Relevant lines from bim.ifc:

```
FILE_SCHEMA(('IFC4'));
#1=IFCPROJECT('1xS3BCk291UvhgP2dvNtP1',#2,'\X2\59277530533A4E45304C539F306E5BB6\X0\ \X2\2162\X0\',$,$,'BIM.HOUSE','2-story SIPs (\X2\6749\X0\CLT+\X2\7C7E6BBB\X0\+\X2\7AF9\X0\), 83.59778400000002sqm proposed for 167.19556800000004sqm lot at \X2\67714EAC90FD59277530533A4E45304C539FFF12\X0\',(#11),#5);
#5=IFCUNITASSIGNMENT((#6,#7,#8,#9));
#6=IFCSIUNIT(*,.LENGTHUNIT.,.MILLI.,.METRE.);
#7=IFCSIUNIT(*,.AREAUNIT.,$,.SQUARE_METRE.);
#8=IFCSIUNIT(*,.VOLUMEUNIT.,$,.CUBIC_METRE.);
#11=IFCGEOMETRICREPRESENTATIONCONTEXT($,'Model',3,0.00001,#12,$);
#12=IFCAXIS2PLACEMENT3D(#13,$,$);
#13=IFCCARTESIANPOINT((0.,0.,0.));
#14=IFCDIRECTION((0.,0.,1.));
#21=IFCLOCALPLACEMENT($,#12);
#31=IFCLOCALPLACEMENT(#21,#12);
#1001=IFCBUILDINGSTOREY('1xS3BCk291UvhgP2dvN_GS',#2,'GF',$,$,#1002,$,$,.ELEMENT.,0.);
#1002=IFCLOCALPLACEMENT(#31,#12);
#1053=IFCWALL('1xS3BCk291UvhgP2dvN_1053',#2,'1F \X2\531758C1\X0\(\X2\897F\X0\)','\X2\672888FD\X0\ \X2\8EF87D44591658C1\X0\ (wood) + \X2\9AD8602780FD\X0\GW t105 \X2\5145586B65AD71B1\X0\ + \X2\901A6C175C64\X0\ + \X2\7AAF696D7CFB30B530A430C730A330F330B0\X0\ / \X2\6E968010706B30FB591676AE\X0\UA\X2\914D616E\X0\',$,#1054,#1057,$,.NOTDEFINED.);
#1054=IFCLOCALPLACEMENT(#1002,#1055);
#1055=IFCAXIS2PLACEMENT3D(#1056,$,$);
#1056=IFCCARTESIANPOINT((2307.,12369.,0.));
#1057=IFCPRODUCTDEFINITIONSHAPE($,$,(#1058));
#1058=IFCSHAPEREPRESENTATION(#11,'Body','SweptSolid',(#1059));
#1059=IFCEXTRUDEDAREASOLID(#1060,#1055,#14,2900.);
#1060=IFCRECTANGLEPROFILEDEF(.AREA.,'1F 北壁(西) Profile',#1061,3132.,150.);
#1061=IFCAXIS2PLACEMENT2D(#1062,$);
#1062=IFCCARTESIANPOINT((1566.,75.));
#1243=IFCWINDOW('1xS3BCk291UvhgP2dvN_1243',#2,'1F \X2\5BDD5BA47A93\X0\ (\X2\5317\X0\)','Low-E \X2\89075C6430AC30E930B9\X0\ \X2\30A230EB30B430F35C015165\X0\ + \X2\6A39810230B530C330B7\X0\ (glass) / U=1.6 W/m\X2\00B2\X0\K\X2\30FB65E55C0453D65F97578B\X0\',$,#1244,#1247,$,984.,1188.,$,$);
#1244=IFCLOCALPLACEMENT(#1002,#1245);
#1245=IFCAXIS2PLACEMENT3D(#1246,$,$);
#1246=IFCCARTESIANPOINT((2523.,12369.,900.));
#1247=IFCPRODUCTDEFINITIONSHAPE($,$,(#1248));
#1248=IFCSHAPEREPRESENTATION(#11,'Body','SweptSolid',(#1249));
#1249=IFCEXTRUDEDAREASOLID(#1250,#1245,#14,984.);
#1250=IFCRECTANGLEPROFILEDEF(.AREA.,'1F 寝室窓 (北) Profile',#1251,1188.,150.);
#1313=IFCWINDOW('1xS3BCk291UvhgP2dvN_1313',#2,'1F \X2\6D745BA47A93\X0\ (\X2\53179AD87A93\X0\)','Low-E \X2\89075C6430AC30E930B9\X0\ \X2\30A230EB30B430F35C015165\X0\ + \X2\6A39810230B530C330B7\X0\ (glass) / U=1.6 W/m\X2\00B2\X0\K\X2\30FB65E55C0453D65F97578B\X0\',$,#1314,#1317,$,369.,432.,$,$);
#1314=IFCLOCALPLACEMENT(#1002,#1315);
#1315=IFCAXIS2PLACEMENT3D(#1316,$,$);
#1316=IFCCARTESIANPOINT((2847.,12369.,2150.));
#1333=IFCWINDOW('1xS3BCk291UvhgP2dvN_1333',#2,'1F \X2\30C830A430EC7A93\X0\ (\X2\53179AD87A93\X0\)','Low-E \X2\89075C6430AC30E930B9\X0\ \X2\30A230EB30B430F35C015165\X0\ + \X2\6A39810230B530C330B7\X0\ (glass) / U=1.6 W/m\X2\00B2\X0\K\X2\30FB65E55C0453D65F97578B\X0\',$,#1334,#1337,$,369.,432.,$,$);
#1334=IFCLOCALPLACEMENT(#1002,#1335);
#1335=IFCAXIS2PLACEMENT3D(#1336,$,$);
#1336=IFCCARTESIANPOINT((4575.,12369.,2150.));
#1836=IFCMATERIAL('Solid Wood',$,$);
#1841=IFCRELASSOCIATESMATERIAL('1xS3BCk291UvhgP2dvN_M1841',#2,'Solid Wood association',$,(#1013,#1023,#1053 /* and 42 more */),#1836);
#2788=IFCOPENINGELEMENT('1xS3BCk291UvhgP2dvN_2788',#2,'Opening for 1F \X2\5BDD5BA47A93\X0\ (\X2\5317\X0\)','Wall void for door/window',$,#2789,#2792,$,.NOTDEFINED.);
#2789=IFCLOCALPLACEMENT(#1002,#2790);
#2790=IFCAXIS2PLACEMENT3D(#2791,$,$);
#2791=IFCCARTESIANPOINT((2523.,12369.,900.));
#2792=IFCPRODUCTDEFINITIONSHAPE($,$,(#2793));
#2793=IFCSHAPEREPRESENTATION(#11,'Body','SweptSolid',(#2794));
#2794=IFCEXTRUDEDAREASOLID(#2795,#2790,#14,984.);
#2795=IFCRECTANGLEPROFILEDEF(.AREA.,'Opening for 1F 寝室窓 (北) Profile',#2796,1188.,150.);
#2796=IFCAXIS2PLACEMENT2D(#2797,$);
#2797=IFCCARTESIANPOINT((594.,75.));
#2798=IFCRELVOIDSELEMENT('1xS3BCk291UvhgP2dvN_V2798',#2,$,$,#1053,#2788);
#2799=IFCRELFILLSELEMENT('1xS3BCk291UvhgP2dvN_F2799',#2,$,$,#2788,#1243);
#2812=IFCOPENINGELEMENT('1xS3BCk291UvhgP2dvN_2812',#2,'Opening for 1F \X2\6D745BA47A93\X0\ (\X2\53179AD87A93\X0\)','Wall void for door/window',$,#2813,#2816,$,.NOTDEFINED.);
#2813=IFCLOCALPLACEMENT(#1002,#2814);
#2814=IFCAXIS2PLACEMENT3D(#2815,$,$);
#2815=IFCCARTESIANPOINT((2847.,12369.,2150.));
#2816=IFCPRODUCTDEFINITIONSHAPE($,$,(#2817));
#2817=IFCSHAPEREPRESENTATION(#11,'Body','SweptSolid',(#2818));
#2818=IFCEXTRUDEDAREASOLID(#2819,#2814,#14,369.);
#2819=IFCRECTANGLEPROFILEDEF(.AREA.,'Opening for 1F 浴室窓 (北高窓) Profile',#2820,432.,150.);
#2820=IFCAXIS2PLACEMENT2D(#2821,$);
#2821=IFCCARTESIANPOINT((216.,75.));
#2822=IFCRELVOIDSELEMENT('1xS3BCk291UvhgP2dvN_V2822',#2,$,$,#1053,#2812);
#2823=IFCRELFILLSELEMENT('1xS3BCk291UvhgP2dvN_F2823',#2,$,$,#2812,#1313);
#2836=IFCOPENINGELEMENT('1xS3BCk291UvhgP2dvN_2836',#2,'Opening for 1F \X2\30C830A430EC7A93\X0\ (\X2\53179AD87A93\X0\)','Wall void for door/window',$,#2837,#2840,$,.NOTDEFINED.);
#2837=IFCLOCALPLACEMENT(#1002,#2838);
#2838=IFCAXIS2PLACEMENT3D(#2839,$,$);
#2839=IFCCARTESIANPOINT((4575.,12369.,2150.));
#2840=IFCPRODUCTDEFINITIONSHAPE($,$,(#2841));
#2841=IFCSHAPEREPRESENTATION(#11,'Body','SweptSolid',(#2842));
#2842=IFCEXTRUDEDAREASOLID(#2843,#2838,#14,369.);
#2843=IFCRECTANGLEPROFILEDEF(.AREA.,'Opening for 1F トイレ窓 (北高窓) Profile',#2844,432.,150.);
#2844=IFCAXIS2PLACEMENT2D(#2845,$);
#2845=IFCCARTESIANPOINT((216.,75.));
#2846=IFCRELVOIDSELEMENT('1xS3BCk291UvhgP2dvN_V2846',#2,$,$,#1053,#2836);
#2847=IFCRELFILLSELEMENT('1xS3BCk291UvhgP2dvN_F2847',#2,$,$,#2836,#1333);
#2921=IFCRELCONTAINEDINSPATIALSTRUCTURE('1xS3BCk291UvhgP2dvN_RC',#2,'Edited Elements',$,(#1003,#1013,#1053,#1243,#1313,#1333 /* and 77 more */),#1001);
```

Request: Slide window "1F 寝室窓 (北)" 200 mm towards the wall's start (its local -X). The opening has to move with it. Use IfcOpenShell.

```python
import ifcopenshell
import ifcopenshell.api.geometry
import ifcopenshell.util.placement
import ifcopenshell.util.unit

model = ifcopenshell.open("bim.ifc")
unit_scale = ifcopenshell.util.unit.calculate_unit_scale(model)

window = model.by_guid("1xS3BCk291UvhgP2dvN_1243")
opening = window.FillsVoids[0].RelatingOpeningElement
wall = opening.VoidsElements[0].RelatingBuildingElement

wall_matrix = ifcopenshell.util.placement.get_local_placement(wall.ObjectPlacement)
shift = wall_matrix[:3, 0] * -0.2 / unit_scale
before = ifcopenshell.util.placement.get_local_placement(window.ObjectPlacement)[:3, 3].copy()

# The window is not placed relative to its opening, so move both.
for product in (opening, window):
    matrix = ifcopenshell.util.placement.get_local_placement(product.ObjectPlacement)
    matrix[:3, 3] += shift
    ifcopenshell.api.geometry.edit_object_placement(model, product=product, matrix=matrix, is_si=False)

after = ifcopenshell.util.placement.get_local_placement(window.ObjectPlacement)[:3, 3]
print("window moved by", (after - before).round(3) + 0.0)

model.write("bim_rev.ifc")
```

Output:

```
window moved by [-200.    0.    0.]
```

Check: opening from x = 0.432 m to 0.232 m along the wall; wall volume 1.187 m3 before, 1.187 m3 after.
